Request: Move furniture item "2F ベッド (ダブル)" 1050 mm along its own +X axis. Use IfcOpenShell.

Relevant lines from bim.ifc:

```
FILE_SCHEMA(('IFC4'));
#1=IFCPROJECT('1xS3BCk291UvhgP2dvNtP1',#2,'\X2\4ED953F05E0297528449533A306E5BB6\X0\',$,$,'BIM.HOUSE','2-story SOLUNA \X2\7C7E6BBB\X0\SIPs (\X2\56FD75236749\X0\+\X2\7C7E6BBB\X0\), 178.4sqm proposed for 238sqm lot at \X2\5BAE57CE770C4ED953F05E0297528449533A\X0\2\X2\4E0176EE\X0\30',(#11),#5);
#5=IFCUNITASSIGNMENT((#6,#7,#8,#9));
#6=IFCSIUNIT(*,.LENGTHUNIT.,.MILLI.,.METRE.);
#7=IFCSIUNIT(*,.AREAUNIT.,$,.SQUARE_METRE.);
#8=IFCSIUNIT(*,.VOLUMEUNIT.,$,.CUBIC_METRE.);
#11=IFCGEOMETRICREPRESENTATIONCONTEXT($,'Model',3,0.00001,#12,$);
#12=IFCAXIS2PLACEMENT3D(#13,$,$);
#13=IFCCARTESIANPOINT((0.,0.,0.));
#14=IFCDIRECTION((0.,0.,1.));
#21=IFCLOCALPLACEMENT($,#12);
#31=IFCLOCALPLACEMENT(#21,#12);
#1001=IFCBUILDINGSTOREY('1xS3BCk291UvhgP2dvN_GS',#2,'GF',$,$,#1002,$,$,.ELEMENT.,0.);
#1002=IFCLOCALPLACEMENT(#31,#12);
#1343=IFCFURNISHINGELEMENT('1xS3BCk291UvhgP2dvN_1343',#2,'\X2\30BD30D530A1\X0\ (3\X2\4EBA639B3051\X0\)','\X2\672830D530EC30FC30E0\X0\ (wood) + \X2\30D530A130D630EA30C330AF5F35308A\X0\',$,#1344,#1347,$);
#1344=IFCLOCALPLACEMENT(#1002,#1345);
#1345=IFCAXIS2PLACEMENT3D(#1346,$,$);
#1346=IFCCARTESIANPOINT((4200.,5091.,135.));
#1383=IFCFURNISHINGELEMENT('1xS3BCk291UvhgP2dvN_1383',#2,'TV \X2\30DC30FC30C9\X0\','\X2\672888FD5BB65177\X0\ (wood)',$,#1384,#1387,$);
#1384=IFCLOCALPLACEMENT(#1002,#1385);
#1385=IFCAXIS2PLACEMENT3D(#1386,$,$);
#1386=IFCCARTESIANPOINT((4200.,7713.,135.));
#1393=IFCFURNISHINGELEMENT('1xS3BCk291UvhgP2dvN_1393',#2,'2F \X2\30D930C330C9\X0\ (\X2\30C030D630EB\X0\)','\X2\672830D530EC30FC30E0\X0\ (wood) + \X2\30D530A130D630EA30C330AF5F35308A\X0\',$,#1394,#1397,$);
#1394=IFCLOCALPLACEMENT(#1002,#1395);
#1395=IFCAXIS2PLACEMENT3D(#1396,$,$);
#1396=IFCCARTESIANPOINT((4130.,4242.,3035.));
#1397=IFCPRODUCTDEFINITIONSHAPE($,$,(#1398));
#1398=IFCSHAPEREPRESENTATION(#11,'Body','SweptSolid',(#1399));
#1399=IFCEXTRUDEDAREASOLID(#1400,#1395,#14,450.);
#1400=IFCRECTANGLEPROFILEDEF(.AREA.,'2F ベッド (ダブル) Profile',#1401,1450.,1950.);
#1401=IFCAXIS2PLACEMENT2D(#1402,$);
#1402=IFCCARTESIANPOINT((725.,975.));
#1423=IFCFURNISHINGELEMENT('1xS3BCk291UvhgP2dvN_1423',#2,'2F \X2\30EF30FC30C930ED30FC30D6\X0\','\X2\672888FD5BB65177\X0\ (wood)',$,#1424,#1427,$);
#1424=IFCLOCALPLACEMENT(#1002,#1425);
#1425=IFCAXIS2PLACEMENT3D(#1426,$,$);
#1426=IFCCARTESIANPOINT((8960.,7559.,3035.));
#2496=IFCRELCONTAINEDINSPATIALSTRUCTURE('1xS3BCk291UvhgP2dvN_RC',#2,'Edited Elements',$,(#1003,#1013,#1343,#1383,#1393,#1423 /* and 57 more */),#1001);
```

```python
import ifcopenshell
import ifcopenshell.api.geometry
import ifcopenshell.util.placement
import ifcopenshell.util.unit

model = ifcopenshell.open("bim.ifc")
unit_scale = ifcopenshell.util.unit.calculate_unit_scale(model)

item = model.by_id(1393)
matrix = ifcopenshell.util.placement.get_local_placement(item.ObjectPlacement)
matrix[:3, 3] += matrix[:3, 0] * 1.05 / unit_scale
ifcopenshell.api.geometry.edit_object_placement(model, product=item, matrix=matrix, is_si=False)

print(ifcopenshell.util.placement.get_local_placement(item.ObjectPlacement).round(3) + 0.0)

model.write("bim_edited.ifc")
```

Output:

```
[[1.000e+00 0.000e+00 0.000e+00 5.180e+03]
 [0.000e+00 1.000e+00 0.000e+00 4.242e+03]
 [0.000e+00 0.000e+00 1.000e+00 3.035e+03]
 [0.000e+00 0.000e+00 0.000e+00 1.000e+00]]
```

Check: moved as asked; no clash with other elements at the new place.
